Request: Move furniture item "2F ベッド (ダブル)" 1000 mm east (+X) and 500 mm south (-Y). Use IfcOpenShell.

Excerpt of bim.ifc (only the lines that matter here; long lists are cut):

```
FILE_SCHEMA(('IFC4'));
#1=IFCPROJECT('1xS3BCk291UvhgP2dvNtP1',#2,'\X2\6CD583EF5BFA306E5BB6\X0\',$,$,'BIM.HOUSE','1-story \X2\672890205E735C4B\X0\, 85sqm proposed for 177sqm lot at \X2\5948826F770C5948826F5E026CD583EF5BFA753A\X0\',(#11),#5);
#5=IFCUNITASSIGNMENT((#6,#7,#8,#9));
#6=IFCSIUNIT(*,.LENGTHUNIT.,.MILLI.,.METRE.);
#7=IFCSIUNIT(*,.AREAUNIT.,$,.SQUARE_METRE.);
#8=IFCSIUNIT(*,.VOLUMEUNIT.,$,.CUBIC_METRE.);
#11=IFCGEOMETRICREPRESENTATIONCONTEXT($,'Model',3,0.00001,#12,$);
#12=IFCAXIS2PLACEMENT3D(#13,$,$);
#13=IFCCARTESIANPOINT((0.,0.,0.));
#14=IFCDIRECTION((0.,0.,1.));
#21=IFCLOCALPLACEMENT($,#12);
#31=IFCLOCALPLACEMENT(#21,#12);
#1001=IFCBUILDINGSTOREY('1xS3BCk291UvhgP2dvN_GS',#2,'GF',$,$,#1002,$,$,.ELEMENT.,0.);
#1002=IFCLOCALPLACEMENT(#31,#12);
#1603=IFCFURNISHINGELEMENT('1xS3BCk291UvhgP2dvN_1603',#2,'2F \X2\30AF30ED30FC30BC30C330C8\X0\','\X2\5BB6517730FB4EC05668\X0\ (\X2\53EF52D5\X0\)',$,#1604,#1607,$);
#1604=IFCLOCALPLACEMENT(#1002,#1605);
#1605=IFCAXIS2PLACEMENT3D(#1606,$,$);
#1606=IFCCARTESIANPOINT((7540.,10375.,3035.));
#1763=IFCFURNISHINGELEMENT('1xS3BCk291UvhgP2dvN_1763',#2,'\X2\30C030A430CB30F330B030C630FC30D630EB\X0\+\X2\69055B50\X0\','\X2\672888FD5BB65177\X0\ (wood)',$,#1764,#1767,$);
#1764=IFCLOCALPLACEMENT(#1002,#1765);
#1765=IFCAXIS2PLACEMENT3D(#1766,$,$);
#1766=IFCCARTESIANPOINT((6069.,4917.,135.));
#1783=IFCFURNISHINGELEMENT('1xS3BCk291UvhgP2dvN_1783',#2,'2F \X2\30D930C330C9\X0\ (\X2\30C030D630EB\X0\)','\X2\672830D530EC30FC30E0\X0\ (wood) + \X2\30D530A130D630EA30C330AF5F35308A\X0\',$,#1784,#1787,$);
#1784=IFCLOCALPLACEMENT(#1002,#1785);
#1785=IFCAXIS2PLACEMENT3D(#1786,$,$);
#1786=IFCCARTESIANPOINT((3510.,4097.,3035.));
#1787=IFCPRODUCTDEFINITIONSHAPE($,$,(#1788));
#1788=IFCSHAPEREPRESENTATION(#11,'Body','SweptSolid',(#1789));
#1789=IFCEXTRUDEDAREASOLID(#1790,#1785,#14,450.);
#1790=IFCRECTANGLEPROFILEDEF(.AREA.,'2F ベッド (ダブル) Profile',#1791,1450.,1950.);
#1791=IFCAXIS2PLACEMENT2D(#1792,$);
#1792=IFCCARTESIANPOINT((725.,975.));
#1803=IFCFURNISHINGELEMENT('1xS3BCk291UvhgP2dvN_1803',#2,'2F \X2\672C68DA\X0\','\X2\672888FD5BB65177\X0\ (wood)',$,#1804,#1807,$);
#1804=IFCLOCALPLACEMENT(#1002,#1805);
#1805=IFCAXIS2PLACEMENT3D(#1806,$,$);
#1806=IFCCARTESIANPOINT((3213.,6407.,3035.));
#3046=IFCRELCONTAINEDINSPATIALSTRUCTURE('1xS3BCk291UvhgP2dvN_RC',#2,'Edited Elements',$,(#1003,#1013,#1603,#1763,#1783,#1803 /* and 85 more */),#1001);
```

```python
import ifcopenshell
import ifcopenshell.api.geometry
import ifcopenshell.util.placement

model = ifcopenshell.open("bim.ifc")

item = model.by_guid("1xS3BCk291UvhgP2dvN_1783")
matrix = ifcopenshell.util.placement.get_local_placement(item.ObjectPlacement)
matrix[0, 3] += 1000.0
matrix[1, 3] -= 500.0
ifcopenshell.api.geometry.edit_object_placement(model, product=item, matrix=matrix, is_si=False)

print(ifcopenshell.util.placement.get_local_placement(item.ObjectPlacement).round(3) + 0.0)

model.write("bim_edited.ifc")
```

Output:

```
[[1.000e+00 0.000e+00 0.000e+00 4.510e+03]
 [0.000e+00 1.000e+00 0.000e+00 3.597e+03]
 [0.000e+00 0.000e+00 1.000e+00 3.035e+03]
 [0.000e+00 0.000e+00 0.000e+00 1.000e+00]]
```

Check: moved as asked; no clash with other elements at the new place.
